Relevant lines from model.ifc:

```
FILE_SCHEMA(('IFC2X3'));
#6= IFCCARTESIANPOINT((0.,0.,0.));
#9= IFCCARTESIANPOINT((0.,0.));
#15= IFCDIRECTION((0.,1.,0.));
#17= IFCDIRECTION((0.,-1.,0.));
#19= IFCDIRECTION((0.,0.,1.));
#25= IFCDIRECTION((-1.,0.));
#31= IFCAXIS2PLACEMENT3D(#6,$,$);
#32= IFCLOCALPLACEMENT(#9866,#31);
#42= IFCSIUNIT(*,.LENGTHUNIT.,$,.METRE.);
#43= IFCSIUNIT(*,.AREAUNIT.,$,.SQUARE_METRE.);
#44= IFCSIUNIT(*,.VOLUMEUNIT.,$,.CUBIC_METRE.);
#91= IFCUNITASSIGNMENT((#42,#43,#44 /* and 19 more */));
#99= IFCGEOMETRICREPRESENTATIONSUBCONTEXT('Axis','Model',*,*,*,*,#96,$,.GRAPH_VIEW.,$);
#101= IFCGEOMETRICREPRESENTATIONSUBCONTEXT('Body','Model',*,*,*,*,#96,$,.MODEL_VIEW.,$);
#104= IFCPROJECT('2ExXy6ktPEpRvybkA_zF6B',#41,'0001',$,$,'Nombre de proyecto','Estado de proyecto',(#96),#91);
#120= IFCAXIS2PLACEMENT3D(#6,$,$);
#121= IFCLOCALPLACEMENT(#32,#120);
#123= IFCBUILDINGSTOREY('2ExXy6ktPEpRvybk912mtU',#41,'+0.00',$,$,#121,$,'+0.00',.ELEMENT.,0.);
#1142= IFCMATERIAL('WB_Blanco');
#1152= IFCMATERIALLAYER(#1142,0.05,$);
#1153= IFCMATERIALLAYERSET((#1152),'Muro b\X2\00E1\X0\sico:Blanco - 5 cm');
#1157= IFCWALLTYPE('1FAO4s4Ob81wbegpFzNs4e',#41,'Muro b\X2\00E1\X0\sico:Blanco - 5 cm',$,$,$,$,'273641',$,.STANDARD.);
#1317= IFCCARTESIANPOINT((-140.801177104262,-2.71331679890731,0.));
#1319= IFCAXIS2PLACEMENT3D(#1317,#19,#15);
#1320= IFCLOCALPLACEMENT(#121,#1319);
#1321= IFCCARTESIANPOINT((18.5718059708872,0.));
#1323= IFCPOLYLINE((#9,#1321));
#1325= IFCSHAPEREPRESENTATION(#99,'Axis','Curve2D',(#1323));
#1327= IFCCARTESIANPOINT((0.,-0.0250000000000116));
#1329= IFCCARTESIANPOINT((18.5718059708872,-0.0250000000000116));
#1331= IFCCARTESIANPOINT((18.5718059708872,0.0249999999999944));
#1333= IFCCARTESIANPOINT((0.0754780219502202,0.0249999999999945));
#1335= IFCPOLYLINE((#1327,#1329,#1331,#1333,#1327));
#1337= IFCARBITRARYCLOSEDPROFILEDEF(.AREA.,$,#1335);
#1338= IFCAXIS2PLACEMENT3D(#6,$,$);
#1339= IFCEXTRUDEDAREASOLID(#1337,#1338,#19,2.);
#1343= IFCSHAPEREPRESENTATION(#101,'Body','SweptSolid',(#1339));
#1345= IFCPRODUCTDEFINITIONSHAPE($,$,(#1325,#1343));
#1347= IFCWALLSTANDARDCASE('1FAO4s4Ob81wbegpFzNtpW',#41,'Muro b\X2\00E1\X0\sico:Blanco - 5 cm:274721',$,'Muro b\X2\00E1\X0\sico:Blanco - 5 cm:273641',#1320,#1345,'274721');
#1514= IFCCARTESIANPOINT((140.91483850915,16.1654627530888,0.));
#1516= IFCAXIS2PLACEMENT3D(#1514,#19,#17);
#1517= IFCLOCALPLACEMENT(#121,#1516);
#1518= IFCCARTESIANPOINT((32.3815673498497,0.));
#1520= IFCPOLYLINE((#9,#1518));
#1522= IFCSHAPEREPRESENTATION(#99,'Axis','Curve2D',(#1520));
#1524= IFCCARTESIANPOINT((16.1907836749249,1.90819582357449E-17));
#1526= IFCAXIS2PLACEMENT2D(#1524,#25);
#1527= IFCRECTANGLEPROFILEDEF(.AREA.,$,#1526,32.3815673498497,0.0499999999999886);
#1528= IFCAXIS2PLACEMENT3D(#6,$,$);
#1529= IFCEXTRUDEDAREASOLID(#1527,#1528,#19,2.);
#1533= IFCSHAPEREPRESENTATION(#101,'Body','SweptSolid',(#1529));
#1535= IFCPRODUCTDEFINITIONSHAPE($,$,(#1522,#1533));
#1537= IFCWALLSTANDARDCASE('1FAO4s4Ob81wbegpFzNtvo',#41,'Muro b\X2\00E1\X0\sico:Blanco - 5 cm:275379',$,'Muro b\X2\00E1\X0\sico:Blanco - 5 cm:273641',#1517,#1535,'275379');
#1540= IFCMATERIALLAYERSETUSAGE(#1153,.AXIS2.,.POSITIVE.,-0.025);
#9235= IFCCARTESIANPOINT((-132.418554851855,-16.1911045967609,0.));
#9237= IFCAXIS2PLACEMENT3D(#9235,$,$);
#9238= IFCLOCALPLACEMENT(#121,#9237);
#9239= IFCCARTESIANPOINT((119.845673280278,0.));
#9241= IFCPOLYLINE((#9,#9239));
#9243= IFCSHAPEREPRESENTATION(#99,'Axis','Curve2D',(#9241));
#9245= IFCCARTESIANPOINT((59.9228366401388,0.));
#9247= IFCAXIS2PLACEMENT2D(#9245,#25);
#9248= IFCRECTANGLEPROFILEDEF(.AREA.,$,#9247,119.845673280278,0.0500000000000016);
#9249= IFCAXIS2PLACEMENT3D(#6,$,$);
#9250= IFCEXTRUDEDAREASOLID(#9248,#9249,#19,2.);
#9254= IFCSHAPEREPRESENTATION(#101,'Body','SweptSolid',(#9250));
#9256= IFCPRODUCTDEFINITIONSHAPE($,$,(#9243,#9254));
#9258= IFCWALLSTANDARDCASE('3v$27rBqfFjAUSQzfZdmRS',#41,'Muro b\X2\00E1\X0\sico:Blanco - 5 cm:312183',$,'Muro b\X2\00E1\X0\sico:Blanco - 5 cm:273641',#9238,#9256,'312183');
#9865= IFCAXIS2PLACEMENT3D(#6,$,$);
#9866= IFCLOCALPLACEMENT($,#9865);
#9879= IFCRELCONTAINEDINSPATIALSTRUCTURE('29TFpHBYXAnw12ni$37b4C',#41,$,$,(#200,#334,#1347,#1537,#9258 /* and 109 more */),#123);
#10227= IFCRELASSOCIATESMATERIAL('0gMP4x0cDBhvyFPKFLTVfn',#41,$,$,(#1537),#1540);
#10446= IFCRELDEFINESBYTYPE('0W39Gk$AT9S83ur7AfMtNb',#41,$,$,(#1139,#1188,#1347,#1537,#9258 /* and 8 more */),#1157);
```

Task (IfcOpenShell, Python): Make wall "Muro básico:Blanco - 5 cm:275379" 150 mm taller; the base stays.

```python
import ifcopenshell
import ifcopenshell.geom
import ifcopenshell.util.representation
import ifcopenshell.util.shape
import ifcopenshell.util.unit

model = ifcopenshell.open("model.ifc")
unit_scale = ifcopenshell.util.unit.calculate_unit_scale(model)
settings = ifcopenshell.geom.settings()


def volume(element):
    """Net volume in cubic metres, openings subtracted."""
    shape = ifcopenshell.geom.create_shape(settings, element)
    return ifcopenshell.util.shape.get_volume(shape.geometry)


wall = model.by_guid("1FAO4s4Ob81wbegpFzNtvo")
before = volume(wall)

body = ifcopenshell.util.representation.get_representation(wall, "Model", "Body")
solid = body.Items[0]
old_height = solid.Depth
solid.Depth += 0.15 / unit_scale
after = volume(wall)

print(f"height {old_height:g} -> {solid.Depth:g}, volume {before:.3f} -> {after:.3f} m3")

model.write("model_v2.ifc")
```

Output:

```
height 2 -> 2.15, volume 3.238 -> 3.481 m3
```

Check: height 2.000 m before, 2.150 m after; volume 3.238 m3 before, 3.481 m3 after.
